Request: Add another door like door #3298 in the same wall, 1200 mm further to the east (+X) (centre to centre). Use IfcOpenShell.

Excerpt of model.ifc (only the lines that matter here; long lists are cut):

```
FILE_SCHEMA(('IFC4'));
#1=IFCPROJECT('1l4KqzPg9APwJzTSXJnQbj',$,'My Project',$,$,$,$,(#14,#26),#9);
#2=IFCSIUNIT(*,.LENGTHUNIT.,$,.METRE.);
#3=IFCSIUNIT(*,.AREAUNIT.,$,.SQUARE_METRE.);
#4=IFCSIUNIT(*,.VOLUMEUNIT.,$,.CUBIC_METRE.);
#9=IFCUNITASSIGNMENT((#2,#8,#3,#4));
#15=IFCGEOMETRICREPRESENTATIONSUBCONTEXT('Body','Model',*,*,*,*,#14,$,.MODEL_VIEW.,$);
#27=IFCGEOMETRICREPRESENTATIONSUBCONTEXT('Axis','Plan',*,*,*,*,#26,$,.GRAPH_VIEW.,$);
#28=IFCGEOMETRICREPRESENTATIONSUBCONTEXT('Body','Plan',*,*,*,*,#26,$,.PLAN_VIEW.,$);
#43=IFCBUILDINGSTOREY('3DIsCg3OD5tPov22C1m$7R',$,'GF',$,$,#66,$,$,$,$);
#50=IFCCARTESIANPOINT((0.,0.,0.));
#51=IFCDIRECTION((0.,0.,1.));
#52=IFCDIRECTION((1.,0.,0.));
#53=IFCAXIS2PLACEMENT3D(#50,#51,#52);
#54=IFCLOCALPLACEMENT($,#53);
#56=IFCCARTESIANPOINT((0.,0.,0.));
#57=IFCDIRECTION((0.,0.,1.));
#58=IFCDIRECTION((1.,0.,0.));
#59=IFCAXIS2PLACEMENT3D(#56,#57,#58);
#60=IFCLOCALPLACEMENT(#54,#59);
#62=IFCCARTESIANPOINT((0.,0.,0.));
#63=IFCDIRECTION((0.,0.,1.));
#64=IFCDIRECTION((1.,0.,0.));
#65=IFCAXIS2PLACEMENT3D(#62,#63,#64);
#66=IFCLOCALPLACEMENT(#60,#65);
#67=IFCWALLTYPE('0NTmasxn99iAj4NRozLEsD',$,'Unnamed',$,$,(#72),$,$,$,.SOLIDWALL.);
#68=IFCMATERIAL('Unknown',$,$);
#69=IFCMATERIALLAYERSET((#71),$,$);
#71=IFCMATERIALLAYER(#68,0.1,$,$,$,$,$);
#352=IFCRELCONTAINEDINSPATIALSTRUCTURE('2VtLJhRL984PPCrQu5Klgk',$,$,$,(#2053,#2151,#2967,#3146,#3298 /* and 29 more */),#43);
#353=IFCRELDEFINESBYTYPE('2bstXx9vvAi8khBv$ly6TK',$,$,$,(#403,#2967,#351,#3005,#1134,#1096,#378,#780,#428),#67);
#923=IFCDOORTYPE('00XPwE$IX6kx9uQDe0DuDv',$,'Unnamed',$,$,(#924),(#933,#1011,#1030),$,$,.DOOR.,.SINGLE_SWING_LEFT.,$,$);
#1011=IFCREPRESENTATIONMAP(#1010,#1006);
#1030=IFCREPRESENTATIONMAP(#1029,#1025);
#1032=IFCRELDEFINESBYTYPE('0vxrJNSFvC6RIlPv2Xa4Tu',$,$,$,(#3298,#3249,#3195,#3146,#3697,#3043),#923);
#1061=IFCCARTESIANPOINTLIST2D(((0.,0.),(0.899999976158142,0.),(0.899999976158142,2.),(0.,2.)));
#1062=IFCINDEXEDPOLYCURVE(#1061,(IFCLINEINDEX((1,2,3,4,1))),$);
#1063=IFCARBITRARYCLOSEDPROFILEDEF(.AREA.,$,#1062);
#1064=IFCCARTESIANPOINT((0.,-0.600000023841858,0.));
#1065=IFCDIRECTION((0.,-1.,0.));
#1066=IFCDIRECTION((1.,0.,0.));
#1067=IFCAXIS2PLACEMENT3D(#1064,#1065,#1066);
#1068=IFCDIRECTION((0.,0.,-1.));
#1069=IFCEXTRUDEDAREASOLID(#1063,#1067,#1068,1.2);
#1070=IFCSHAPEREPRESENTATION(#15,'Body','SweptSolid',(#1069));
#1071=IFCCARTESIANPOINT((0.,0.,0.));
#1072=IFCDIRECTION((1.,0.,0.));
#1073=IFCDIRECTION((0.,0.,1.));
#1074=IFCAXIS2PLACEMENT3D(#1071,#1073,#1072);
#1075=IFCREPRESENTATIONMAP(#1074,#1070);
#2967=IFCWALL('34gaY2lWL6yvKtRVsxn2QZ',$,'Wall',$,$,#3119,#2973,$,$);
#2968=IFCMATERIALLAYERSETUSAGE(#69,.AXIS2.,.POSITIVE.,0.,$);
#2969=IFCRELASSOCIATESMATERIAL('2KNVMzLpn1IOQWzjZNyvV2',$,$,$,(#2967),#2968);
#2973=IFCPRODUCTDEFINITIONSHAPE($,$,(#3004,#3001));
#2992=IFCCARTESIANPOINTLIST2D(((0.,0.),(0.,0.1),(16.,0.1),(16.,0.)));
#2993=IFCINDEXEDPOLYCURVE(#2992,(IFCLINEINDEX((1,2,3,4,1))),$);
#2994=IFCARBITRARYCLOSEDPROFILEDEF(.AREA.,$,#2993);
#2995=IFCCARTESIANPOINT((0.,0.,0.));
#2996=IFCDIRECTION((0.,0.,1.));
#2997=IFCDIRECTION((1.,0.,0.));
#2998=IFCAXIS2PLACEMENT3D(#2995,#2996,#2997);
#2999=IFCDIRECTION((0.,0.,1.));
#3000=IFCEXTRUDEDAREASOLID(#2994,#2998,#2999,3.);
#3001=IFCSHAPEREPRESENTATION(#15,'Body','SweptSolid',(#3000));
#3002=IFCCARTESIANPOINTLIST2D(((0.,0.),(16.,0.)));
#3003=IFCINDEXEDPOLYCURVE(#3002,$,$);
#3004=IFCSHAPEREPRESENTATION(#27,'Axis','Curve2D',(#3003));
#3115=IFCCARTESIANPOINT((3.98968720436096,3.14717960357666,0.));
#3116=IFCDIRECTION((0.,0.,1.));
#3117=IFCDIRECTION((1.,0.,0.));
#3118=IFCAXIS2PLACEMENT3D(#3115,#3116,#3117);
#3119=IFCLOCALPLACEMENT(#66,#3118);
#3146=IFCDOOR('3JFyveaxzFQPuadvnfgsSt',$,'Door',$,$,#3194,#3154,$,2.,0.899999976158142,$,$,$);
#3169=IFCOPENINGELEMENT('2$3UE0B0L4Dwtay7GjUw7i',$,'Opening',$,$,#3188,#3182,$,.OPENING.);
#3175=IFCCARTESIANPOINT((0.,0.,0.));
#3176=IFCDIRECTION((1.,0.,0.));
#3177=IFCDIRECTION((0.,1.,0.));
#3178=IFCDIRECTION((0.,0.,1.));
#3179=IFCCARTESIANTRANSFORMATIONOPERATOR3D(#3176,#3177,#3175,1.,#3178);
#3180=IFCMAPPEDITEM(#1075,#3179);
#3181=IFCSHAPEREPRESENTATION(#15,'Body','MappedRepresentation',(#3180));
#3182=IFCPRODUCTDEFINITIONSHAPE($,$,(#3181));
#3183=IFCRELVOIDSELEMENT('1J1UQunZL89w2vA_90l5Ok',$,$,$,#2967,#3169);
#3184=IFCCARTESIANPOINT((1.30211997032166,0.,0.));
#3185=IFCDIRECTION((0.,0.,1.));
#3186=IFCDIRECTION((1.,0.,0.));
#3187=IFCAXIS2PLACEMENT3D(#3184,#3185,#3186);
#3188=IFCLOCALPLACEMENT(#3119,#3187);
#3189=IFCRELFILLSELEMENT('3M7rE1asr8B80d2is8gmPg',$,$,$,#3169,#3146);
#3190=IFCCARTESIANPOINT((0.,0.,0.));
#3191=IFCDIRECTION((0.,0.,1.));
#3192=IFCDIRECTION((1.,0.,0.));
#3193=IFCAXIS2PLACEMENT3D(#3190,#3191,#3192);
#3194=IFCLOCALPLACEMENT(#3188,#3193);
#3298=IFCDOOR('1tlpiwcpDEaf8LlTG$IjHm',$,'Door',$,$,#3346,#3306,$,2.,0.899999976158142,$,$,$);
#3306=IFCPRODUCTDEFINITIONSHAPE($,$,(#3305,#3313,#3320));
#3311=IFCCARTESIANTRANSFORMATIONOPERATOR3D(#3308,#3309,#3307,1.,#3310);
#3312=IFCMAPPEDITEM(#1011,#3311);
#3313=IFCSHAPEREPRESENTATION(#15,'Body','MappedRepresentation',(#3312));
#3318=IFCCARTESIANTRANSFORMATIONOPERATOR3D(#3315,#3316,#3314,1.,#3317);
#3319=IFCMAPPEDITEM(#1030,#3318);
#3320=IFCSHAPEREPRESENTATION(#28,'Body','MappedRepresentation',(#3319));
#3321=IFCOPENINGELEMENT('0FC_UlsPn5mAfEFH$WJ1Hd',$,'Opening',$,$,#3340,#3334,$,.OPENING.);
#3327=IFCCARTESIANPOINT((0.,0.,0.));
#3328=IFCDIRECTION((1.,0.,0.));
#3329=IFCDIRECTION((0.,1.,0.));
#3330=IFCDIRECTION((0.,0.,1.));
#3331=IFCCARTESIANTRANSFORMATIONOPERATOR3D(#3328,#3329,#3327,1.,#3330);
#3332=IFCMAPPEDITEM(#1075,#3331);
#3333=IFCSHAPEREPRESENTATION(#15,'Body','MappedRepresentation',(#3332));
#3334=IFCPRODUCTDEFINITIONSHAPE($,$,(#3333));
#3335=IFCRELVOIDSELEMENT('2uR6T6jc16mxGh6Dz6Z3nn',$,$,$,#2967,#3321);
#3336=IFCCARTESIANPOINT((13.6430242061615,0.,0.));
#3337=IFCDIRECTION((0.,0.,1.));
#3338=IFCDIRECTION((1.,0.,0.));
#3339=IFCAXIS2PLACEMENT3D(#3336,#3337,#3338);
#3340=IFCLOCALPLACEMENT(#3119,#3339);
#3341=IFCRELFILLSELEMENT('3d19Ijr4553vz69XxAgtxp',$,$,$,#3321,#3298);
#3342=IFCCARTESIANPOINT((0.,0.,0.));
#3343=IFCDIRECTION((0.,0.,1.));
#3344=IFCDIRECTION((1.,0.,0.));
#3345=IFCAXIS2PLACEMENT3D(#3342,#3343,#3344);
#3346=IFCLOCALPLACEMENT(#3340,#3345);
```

```python
import ifcopenshell
import ifcopenshell.api.feature
import ifcopenshell.api.geometry
import ifcopenshell.api.root
import ifcopenshell.geom
import ifcopenshell.util.element
import ifcopenshell.util.placement
import ifcopenshell.util.shape
import ifcopenshell.util.unit

model = ifcopenshell.open("model.ifc")
unit_scale = ifcopenshell.util.unit.calculate_unit_scale(model)
settings = ifcopenshell.geom.settings()


def volume(element):
    """Net volume in cubic metres, openings subtracted."""
    shape = ifcopenshell.geom.create_shape(settings, element)
    return ifcopenshell.util.shape.get_volume(shape.geometry)


door = model.by_guid("1tlpiwcpDEaf8LlTG$IjHm")
opening = door.FillsVoids[0].RelatingOpeningElement
wall = opening.VoidsElements[0].RelatingBuildingElement
before = volume(wall)
shift = ifcopenshell.util.placement.get_local_placement(wall.ObjectPlacement)[:3, 0] * 1.2 / unit_scale

# copy_class copies the void relationship, type, container and properties, but no geometry.
new_opening = ifcopenshell.api.root.copy_class(model, product=opening)
new_opening.Representation = ifcopenshell.util.element.copy_deep(
    model, opening.Representation, exclude=["IfcGeometricRepresentationContext", "IfcRepresentationMap"]
)
new_door = ifcopenshell.api.root.copy_class(model, product=door)
new_door.Representation = ifcopenshell.util.element.copy_deep(
    model, door.Representation, exclude=["IfcGeometricRepresentationContext", "IfcRepresentationMap"]
)
ifcopenshell.api.feature.add_filling(model, opening=new_opening, element=new_door)

for old, new in ((opening, new_opening), (door, new_door)):
    matrix = ifcopenshell.util.placement.get_local_placement(old.ObjectPlacement)
    matrix[:3, 3] += shift
    ifcopenshell.api.geometry.edit_object_placement(model, product=new, matrix=matrix, is_si=False)

after = volume(wall)

print(f"wall volume {before:.3f} -> {after:.3f} m3")

model.write("model-out.ifc")
```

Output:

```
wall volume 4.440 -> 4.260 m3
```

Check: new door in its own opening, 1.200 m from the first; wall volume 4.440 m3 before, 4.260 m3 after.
